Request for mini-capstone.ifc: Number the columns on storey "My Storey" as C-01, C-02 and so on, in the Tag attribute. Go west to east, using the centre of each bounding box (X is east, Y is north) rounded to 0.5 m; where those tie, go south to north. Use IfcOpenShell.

First a look at what the model holds.

```python
import ifcopenshell
import ifcopenshell.util.element
import ifcopenshell.util.placement

model = ifcopenshell.open("mini-capstone.ifc")
print(model.schema)
storey = next(s for s in model.by_type("IfcBuildingStorey") if s.Name == "My Storey")
columns = [e for e in ifcopenshell.util.element.get_decomposition(storey) if e.is_a("IfcColumn")]
for e in sorted(columns, key=lambda e: e.id()):
    origin = ifcopenshell.util.placement.get_local_placement(e.ObjectPlacement)[:3, 3]
    print(e.id(), e.Tag, e.Name, origin.round(2) + 0.0, sep=" | ")
```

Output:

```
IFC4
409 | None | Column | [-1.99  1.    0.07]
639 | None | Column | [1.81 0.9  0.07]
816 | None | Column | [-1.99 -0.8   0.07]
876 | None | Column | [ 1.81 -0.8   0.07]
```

```python
import ifcopenshell
import ifcopenshell.geom
import ifcopenshell.util.element
import ifcopenshell.util.shape

model = ifcopenshell.open("mini-capstone.ifc")
settings = ifcopenshell.geom.settings()
settings.set("use-world-coords", True)


def centre(element):
    shape = ifcopenshell.geom.create_shape(settings, element)
    return ifcopenshell.util.shape.get_bbox_centroid(shape.geometry)


storey = next(s for s in model.by_type("IfcBuildingStorey") if s.Name == "My Storey")
columns = [e for e in ifcopenshell.util.element.get_decomposition(storey) if e.is_a("IfcColumn")]

# Insertion points can sit at a corner or the storey origin, so sort by the geometry (in metres).
centres = {e: centre(e) for e in columns}
columns.sort(key=lambda e: (round(centres[e][0] / 0.5), centres[e][1]))

for i, e in enumerate(columns, start=1):
    number = f"C-{i:02d}"
    e.Tag = number
    print(e.id(), number)

model.write("mini-capstone_updated.ifc")
```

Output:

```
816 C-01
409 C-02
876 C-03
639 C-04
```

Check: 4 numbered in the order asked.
